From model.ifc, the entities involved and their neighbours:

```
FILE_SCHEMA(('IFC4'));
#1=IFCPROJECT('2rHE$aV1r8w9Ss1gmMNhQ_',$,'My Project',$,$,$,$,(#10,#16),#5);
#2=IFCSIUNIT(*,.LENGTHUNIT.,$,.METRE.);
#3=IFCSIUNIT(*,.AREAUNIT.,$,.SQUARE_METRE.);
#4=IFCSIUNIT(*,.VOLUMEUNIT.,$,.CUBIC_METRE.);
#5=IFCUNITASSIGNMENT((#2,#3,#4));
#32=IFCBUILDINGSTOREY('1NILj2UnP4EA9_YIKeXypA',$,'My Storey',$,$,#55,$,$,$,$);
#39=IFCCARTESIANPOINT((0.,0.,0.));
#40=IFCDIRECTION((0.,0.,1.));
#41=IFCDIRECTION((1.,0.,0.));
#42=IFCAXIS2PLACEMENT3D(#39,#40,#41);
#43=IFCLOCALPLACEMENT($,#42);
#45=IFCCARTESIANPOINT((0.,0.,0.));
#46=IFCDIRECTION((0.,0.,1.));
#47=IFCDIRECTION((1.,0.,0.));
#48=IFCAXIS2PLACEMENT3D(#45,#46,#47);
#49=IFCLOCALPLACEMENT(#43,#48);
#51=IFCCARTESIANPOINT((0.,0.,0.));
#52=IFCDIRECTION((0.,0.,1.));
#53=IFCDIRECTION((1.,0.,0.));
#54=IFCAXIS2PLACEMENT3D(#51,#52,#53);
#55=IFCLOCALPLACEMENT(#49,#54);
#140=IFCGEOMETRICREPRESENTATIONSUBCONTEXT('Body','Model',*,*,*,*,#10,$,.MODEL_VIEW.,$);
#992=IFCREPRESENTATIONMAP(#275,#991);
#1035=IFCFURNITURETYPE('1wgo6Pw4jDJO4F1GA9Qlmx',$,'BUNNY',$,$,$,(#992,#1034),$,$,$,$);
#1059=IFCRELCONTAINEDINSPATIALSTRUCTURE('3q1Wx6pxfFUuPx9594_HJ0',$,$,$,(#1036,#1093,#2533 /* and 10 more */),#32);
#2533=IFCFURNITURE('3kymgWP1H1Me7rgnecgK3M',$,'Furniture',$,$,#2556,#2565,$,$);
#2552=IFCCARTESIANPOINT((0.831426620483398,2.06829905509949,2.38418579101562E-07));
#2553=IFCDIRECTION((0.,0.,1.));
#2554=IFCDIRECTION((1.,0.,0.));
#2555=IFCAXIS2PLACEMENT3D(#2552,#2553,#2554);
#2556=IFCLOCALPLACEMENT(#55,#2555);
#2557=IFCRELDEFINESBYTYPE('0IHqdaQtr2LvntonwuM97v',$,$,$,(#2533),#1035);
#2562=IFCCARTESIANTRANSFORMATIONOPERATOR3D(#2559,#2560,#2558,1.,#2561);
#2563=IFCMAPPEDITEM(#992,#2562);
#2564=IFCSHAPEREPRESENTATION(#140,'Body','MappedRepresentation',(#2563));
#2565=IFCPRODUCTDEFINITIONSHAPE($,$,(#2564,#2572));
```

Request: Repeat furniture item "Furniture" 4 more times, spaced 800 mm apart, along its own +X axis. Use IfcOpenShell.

```python
import ifcopenshell
import ifcopenshell.api.geometry
import ifcopenshell.api.root
import ifcopenshell.util.element
import ifcopenshell.util.placement

model = ifcopenshell.open("model.ifc")

source = model.by_guid("3kymgWP1H1Me7rgnecgK3M")
base = ifcopenshell.util.placement.get_local_placement(source.ObjectPlacement)
step = base[:3, 0] * 0.8

for i in range(1, 5):
    copy = ifcopenshell.api.root.copy_class(model, product=source)
    copy.Representation = ifcopenshell.util.element.copy_deep(
        model, source.Representation, exclude=["IfcGeometricRepresentationContext", "IfcRepresentationMap"]
    )
    matrix = base.copy()
    matrix[:3, 3] += i * step
    print("added at", matrix[:3, 3].round(3) + 0.0)
    ifcopenshell.api.geometry.edit_object_placement(model, product=copy, matrix=matrix, is_si=False)

model.write("model_rev.ifc")
```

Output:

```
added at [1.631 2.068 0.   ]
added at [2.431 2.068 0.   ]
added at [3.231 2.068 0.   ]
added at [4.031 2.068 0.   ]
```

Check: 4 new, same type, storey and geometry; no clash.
